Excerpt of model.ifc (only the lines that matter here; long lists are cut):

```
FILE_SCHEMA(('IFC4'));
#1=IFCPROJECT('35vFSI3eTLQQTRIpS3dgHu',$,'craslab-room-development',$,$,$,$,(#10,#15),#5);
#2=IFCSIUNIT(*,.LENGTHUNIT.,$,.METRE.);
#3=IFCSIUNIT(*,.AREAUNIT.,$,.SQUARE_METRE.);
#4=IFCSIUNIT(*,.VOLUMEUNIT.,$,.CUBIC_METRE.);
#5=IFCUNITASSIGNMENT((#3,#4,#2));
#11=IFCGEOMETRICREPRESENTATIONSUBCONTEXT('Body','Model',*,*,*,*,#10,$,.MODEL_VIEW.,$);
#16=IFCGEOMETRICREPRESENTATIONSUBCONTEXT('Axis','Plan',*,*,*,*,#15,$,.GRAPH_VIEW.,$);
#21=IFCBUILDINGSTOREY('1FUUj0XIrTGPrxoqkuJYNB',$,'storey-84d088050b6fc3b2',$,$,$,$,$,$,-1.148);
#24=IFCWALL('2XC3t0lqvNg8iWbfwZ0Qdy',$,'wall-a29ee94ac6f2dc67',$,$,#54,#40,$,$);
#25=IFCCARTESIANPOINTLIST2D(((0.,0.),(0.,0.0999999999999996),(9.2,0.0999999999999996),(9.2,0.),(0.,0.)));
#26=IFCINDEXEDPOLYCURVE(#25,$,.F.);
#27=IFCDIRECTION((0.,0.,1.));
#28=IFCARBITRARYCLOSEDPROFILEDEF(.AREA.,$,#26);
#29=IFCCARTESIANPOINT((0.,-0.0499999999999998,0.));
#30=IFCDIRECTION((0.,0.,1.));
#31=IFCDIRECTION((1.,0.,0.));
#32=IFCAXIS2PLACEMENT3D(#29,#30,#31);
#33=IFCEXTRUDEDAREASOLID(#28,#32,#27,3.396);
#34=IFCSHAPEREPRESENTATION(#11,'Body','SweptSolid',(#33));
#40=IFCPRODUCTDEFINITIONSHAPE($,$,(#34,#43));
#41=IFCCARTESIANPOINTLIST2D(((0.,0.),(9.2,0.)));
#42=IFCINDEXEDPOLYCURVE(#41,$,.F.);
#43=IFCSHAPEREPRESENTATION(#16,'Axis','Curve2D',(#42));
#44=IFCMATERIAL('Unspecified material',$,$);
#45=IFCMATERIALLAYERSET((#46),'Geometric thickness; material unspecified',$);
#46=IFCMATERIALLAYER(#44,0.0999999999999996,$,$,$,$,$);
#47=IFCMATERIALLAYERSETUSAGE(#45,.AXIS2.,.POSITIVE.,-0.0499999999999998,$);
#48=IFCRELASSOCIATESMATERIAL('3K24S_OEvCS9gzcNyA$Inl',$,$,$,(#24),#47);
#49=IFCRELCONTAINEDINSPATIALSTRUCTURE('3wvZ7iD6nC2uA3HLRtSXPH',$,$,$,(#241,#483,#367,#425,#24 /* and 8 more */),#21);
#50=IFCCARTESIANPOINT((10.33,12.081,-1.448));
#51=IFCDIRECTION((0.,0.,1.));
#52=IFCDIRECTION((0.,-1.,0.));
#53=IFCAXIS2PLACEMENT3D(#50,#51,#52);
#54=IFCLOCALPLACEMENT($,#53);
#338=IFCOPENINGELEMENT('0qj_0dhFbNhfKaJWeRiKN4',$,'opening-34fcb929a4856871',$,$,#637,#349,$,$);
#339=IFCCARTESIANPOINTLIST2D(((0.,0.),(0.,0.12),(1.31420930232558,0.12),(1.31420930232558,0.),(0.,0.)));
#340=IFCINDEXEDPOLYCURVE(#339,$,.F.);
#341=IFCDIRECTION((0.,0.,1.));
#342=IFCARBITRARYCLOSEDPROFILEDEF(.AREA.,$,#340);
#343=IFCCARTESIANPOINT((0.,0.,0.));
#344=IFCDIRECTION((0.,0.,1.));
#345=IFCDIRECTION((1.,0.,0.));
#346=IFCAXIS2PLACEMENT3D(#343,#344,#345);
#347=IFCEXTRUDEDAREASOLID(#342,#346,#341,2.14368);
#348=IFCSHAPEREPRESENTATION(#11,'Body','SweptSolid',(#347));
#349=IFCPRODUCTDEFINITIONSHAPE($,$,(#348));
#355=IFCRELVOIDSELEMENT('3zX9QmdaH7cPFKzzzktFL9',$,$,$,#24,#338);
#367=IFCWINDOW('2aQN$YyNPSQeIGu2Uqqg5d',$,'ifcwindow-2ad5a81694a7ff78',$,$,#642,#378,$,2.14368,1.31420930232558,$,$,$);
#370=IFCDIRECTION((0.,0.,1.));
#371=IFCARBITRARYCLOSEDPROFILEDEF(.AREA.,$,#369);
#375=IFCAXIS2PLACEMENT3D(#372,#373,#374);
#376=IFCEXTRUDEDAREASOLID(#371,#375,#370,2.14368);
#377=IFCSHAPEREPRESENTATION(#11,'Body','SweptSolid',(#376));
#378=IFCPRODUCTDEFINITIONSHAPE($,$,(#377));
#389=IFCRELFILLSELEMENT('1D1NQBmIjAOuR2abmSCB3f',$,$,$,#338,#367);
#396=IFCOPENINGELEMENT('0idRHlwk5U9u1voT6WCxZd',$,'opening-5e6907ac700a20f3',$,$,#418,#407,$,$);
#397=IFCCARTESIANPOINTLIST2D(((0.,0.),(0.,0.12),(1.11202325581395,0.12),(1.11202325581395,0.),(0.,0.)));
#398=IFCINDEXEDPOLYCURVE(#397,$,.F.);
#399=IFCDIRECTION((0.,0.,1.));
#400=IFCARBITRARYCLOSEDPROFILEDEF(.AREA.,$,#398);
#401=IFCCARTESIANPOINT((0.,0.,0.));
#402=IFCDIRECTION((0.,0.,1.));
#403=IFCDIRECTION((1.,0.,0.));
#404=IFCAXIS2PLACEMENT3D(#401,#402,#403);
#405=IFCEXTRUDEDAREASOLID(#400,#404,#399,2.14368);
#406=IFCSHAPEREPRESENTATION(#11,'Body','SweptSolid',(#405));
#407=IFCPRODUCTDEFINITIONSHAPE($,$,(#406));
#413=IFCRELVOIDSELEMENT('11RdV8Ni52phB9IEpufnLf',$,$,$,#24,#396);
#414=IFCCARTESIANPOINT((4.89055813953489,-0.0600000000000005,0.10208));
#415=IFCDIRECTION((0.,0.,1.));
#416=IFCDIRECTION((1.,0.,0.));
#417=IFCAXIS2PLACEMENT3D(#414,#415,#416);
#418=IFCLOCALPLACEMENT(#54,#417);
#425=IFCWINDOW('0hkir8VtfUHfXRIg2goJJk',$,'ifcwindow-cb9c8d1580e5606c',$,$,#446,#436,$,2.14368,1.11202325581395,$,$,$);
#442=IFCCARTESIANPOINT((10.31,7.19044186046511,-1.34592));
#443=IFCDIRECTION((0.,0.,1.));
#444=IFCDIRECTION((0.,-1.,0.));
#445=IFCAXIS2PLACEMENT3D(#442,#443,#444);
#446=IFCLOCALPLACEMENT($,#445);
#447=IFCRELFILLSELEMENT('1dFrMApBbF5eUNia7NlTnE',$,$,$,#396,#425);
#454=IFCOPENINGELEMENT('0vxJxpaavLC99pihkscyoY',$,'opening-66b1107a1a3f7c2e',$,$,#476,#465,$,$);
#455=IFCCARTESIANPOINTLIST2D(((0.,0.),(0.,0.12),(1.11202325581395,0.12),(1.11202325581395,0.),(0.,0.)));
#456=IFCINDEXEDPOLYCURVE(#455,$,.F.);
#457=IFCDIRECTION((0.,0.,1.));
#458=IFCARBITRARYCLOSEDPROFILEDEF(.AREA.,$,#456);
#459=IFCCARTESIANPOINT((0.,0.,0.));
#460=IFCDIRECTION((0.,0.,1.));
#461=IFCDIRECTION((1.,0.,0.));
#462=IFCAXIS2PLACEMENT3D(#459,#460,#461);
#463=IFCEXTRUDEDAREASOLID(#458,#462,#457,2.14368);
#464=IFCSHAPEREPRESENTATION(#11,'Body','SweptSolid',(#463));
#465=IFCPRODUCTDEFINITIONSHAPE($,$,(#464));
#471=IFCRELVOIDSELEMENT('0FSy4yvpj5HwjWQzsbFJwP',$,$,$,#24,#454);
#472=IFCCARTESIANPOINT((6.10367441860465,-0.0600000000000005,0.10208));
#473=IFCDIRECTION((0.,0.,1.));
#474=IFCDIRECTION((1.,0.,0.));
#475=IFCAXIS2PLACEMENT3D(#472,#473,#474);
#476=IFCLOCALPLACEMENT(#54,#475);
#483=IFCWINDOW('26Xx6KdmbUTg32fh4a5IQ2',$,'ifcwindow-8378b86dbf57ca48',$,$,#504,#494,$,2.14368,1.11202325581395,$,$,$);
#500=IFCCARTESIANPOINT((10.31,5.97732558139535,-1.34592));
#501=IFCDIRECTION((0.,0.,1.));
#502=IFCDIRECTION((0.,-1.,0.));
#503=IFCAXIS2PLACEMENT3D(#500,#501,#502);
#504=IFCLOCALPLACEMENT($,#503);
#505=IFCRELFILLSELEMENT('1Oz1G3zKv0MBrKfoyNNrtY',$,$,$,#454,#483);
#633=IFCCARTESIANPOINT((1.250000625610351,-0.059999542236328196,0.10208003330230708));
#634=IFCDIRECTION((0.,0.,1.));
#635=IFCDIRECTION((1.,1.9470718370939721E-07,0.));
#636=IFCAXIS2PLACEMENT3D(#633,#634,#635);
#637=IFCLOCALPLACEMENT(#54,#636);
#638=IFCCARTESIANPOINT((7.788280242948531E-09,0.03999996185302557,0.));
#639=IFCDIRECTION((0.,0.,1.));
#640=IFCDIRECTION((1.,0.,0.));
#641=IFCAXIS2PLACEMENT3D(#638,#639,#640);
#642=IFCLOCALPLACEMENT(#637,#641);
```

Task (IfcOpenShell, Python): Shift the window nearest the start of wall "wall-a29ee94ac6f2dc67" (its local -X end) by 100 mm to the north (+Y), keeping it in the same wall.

```python
import ifcopenshell
import ifcopenshell.api.geometry
import ifcopenshell.util.placement
import ifcopenshell.util.unit

model = ifcopenshell.open("model.ifc")
unit_scale = ifcopenshell.util.unit.calculate_unit_scale(model)

window = model.by_guid("2aQN$YyNPSQeIGu2Uqqg5d")
opening = window.FillsVoids[0].RelatingOpeningElement
wall = opening.VoidsElements[0].RelatingBuildingElement

wall_matrix = ifcopenshell.util.placement.get_local_placement(wall.ObjectPlacement)
shift = wall_matrix[:3, 0] * -0.1 / unit_scale
before = ifcopenshell.util.placement.get_local_placement(window.ObjectPlacement)[:3, 3].copy()

# The window is placed relative to its opening, so it follows when the opening moves.
matrix = ifcopenshell.util.placement.get_local_placement(opening.ObjectPlacement)
matrix[:3, 3] += shift
ifcopenshell.api.geometry.edit_object_placement(
    model, product=opening, matrix=matrix, is_si=False, should_transform_children=True
)

after = ifcopenshell.util.placement.get_local_placement(window.ObjectPlacement)[:3, 3]
print("window moved by", (after - before).round(3) + 0.0)

model.write("model_rev.ifc")
```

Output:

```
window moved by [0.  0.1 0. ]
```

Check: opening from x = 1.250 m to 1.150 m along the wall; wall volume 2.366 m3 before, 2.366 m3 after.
